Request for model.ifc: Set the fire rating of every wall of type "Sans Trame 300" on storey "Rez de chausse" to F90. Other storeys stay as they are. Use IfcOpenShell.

First a look at what the model holds.

```python
import ifcopenshell
import ifcopenshell.util.element

model = ifcopenshell.open("model.ifc")
print(model.schema)
storey = next(s for s in model.by_type("IfcBuildingStorey") if s.Name == 'Rez de chauss\x8ee')
walls = [e for e in ifcopenshell.util.element.get_decomposition(storey) if e.is_a("IfcWall")]
seen = {}
for e in walls:
    element_type = ifcopenshell.util.element.get_type(e)
    key = (element_type.Name if element_type != e and element_type else None, ifcopenshell.util.element.get_pset(e, "Pset_WallCommon", "FireRating"))
    seen[key] = seen.get(key, 0) + 1
for (name, value), count in sorted(seen.items(), key=str):
    print(count, "x", name, "|", value)
```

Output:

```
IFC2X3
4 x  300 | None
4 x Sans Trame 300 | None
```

```python
import ifcopenshell
import ifcopenshell.api.pset
import ifcopenshell.util.element

model = ifcopenshell.open("model.ifc")

storey = next(s for s in model.by_type("IfcBuildingStorey") if s.Name == 'Rez de chauss\x8ee')
walls = [e for e in ifcopenshell.util.element.get_decomposition(storey) if e.is_a("IfcWall")]

count = 0
for e in walls:
    element_type = ifcopenshell.util.element.get_type(e)
    if element_type in (None, e) or element_type.Name != "Sans Trame 300":
        continue
    # add_pset returns the element's existing set when there is one.
    pset = ifcopenshell.api.pset.add_pset(model, product=e, name="Pset_WallCommon")
    ifcopenshell.api.pset.edit_pset(model, pset=pset, properties={"FireRating": "F90"})
    count += 1

print(count, "walls updated")

model.write("model-out.ifc")
```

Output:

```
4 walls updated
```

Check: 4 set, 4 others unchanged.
